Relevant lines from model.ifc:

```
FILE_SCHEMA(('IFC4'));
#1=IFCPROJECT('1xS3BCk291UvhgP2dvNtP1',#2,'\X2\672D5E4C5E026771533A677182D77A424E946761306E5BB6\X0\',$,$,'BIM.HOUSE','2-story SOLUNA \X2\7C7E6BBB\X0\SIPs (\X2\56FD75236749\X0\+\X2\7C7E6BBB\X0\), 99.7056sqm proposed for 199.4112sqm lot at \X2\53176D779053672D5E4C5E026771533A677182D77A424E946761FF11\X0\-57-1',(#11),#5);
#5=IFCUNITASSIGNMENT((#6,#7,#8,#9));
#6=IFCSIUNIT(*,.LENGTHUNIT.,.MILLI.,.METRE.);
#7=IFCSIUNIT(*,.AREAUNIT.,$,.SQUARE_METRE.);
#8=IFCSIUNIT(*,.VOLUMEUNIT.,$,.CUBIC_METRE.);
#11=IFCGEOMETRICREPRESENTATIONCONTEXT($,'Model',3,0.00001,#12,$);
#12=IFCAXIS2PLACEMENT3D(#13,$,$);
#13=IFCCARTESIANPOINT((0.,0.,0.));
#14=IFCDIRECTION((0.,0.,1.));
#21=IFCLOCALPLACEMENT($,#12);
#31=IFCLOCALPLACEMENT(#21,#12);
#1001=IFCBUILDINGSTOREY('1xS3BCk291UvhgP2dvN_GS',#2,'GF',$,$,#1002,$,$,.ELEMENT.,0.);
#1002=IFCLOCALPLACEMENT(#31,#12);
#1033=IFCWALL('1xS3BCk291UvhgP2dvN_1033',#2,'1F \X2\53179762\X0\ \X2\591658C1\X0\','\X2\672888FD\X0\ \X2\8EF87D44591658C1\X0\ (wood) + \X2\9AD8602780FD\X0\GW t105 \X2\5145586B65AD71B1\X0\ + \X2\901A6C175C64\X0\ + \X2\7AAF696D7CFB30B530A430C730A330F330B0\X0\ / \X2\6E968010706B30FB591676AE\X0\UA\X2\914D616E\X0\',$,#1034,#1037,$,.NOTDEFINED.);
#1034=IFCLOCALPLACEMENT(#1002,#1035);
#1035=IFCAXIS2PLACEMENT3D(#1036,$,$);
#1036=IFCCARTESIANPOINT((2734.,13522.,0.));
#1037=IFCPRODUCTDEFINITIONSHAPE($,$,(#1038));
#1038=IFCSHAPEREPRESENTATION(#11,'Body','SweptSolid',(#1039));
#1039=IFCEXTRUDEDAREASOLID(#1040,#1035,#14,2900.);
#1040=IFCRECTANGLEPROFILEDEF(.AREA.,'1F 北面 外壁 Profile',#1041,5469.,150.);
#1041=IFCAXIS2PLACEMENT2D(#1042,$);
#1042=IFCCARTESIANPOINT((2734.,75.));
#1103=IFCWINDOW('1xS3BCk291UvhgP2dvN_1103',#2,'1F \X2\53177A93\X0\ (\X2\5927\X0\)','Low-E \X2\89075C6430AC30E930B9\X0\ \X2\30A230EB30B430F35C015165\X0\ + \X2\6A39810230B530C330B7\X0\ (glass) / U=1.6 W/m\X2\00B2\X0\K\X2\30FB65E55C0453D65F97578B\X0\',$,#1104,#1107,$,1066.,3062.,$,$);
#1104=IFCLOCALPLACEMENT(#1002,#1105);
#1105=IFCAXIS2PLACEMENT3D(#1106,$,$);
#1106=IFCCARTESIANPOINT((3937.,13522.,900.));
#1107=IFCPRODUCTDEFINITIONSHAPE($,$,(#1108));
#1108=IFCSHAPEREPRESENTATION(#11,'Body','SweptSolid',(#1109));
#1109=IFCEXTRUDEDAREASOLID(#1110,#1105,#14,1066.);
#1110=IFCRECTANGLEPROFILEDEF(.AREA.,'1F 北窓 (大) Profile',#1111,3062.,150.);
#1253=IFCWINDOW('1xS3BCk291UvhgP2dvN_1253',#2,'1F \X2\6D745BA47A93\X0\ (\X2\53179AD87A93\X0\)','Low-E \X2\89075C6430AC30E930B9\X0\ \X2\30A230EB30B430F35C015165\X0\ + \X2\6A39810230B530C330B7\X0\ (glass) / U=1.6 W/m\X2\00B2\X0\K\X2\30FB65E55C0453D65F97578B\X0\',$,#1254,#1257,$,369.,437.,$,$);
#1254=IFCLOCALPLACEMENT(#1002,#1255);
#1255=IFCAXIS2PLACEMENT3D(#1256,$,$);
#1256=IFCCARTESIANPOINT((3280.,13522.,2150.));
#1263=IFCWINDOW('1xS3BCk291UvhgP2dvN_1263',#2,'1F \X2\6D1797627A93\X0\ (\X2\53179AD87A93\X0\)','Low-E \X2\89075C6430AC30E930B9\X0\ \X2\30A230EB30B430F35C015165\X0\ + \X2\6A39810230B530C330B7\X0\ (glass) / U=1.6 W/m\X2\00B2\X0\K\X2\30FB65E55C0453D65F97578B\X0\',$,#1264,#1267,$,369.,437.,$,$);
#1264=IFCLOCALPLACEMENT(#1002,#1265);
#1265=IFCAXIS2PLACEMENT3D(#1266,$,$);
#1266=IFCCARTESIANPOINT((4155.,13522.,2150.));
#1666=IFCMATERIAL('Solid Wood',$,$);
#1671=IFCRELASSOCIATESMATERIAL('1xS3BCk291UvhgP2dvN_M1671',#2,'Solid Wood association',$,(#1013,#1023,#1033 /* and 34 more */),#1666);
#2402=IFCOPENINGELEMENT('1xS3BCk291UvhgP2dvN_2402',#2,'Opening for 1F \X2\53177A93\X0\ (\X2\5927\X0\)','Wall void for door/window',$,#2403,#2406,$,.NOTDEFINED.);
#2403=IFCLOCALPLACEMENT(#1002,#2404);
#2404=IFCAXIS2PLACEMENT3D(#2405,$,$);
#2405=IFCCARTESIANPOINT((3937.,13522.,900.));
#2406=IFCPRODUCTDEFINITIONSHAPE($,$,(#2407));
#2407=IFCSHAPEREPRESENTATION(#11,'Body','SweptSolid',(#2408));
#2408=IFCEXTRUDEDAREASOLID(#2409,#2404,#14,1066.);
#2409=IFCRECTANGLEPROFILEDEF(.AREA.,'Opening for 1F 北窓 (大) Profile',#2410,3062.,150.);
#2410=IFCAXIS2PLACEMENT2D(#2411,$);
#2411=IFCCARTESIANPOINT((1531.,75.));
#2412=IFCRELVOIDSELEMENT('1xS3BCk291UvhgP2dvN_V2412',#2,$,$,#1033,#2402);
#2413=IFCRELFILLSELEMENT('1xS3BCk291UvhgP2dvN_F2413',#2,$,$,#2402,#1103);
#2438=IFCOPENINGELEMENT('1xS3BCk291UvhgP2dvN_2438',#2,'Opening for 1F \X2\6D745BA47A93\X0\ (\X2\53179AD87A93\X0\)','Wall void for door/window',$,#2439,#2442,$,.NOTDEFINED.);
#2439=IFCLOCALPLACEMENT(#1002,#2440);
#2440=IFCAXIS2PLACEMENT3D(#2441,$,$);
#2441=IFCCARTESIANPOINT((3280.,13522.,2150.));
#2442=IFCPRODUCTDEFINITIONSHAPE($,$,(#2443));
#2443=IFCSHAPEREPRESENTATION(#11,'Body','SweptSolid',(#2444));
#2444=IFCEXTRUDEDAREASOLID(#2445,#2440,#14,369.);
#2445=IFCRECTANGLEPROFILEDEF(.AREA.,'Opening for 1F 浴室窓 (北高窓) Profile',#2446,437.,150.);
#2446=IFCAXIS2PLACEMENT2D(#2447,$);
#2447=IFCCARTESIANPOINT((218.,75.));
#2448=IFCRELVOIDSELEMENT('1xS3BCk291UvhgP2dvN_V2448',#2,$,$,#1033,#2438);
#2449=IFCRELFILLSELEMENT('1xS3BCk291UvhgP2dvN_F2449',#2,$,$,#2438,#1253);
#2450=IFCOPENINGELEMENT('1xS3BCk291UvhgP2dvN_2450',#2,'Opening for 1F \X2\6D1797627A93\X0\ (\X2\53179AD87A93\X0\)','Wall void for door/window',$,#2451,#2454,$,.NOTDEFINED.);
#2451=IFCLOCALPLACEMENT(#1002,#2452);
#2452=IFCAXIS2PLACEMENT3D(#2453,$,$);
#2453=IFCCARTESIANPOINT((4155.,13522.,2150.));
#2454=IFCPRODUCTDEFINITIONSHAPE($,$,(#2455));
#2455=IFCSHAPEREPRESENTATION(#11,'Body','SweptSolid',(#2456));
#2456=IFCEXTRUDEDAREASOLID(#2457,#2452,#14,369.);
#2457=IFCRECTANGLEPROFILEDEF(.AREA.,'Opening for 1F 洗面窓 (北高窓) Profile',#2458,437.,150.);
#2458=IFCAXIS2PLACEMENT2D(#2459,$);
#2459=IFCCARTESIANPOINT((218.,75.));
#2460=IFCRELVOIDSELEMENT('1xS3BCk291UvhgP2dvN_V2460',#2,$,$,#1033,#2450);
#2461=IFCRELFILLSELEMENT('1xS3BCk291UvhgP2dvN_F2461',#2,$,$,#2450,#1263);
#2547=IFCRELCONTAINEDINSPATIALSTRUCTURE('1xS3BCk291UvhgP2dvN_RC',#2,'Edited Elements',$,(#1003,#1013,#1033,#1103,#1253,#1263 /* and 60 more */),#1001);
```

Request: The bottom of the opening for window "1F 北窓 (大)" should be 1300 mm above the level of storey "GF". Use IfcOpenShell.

```python
import numpy as np
import ifcopenshell
import ifcopenshell.api.geometry
import ifcopenshell.geom
import ifcopenshell.util.element
import ifcopenshell.util.placement
import ifcopenshell.util.shape
import ifcopenshell.util.unit

model = ifcopenshell.open("model.ifc")
unit_scale = ifcopenshell.util.unit.calculate_unit_scale(model)

window = model.by_id(1103)
opening = window.FillsVoids[0].RelatingOpeningElement
storey = ifcopenshell.util.element.get_container(window, ifc_class="IfcBuildingStorey")
level = ifcopenshell.util.placement.get_local_placement(storey.ObjectPlacement)[2, 3]

# The opening's origin need not be at the sill, so measure its lowest point.
shape = ifcopenshell.geom.create_shape(ifcopenshell.geom.settings(), opening)
bottom = ifcopenshell.util.shape.get_shape_bottom_elevation(shape, shape.geometry) / unit_scale
dz = level + 1300.0 - bottom

shift = np.array([0.0, 0.0, dz])
# The window is not placed relative to its opening, so move both.
for product in (opening, window):
    matrix = ifcopenshell.util.placement.get_local_placement(product.ObjectPlacement)
    matrix[:3, 3] += shift
    ifcopenshell.api.geometry.edit_object_placement(model, product=product, matrix=matrix, is_si=False)

print(f"moved by {dz * unit_scale:+.3f} m")

model.write("model_rev.ifc")
```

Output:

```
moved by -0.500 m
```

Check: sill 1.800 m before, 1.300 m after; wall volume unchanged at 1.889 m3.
